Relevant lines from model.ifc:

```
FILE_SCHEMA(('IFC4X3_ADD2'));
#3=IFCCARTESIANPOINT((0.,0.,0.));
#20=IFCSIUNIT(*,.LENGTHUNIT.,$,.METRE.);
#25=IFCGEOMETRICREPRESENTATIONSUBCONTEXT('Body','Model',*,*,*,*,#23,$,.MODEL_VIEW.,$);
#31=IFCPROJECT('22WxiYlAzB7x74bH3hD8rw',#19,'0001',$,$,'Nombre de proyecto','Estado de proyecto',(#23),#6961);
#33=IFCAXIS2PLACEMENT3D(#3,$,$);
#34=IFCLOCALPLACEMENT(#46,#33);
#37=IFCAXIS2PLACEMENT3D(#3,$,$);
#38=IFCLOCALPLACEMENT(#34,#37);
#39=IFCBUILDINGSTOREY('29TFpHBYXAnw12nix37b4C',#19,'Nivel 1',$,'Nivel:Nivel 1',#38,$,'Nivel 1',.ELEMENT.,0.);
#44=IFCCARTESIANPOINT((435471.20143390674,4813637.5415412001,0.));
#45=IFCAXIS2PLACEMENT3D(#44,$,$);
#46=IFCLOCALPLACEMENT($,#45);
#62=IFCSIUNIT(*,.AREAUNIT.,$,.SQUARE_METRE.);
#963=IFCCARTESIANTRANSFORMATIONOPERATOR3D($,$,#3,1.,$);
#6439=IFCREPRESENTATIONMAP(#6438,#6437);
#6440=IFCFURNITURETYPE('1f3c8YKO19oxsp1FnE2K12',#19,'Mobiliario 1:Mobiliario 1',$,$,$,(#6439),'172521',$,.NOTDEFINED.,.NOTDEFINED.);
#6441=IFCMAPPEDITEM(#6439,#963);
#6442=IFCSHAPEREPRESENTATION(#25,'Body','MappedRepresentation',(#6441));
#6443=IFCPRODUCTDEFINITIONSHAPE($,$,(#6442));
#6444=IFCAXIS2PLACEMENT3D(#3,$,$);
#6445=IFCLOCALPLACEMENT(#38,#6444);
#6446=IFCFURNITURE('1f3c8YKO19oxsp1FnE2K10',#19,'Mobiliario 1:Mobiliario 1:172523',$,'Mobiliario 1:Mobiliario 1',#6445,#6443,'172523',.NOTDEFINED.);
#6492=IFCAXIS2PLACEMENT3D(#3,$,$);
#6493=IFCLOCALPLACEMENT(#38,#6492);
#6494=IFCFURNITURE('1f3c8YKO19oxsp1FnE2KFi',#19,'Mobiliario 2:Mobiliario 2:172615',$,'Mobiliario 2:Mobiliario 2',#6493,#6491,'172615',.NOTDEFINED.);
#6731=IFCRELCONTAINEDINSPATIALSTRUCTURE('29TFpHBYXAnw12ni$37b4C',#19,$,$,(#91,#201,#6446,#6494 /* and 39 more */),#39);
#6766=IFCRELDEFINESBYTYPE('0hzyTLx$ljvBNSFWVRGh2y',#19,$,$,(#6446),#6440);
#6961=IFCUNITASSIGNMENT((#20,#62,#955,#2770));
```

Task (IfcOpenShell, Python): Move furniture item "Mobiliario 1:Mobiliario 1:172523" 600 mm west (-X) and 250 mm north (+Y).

```python
import ifcopenshell
import ifcopenshell.api.geometry
import ifcopenshell.util.placement
import ifcopenshell.util.unit

model = ifcopenshell.open("model.ifc")
unit_scale = ifcopenshell.util.unit.calculate_unit_scale(model)

item = model.by_guid("1f3c8YKO19oxsp1FnE2K10")
matrix = ifcopenshell.util.placement.get_local_placement(item.ObjectPlacement)
matrix[0, 3] -= 0.6 / unit_scale
matrix[1, 3] += 0.25 / unit_scale
ifcopenshell.api.geometry.edit_object_placement(model, product=item, matrix=matrix, is_si=False)

print(ifcopenshell.util.placement.get_local_placement(item.ObjectPlacement).round(3) + 0.0)

model.write("model_v2.ifc")
```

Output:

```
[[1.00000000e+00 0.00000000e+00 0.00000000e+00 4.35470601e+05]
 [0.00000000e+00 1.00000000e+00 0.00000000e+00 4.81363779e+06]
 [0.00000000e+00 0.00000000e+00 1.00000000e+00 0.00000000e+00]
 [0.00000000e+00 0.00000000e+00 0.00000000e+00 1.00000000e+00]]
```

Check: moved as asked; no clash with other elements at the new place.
